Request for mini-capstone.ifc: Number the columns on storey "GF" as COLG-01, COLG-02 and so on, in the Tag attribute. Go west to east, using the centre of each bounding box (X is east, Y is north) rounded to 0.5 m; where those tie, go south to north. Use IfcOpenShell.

First a look at what the model holds.

```python
import ifcopenshell
import ifcopenshell.util.element
import ifcopenshell.util.placement

model = ifcopenshell.open("mini-capstone.ifc")
print(model.schema)
storey = next(s for s in model.by_type("IfcBuildingStorey") if s.Name == "GF")
columns = [e for e in ifcopenshell.util.element.get_decomposition(storey) if e.is_a("IfcColumn")]
for e in sorted(columns, key=lambda e: e.id()):
    origin = ifcopenshell.util.placement.get_local_placement(e.ObjectPlacement)[:3, 3]
    print(e.id(), e.Tag, e.Name, origin.round(2) + 0.0, sep=" | ")
```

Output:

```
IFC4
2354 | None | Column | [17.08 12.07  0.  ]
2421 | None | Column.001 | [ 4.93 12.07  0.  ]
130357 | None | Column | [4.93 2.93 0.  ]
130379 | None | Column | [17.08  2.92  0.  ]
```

```python
import ifcopenshell
import ifcopenshell.geom
import ifcopenshell.util.element
import ifcopenshell.util.shape

model = ifcopenshell.open("mini-capstone.ifc")
settings = ifcopenshell.geom.settings()
settings.set("use-world-coords", True)


def centre(element):
    shape = ifcopenshell.geom.create_shape(settings, element)
    return ifcopenshell.util.shape.get_bbox_centroid(shape.geometry)


storey = next(s for s in model.by_type("IfcBuildingStorey") if s.Name == "GF")
columns = [e for e in ifcopenshell.util.element.get_decomposition(storey) if e.is_a("IfcColumn")]

# Insertion points can sit at a corner or the storey origin, so sort by the geometry (in metres).
centres = {e: centre(e) for e in columns}
columns.sort(key=lambda e: (round(centres[e][0] / 0.5), centres[e][1]))

for i, e in enumerate(columns, start=1):
    number = f"COLG-{i:02d}"
    e.Tag = number
    print(e.id(), number)

model.write("mini-capstone_edited.ifc")
```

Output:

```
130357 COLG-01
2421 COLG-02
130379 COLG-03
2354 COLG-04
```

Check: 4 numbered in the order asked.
